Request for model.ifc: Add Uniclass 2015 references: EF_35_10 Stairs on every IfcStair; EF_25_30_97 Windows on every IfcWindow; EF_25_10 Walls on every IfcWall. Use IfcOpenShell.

First a look at what the model holds.

```python
import ifcopenshell

model = ifcopenshell.open("model.ifc")
print(model.schema)
print("classifications:", [c.Name for c in model.by_type("IfcClassification")])
for ifc_class in ("IfcDoor", "IfcRoof", "IfcStair", "IfcWall", "IfcWindow"):
    print(ifc_class, len(model.by_type(ifc_class)))
```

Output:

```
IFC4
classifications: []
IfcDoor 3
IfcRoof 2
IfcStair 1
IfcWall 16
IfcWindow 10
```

```python
import ifcopenshell
import ifcopenshell.api.classification

model = ifcopenshell.open("model.ifc")

system = ifcopenshell.api.classification.add_classification(model, classification="Uniclass 2015")

codes = {
    "IfcStair": ("EF_35_10", "Stairs"),
    "IfcWindow": ("EF_25_30_97", "Windows"),
    "IfcWall": ("EF_25_10", "Walls"),
}
for ifc_class, (code, name) in codes.items():
    products = model.by_type(ifc_class)
    ifcopenshell.api.classification.add_reference(
        model, products=products, classification=system, identification=code, name=name
    )
    print(code, len(products))

model.write("model_v2.ifc")
```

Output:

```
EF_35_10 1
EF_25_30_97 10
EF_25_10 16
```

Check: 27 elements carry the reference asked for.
